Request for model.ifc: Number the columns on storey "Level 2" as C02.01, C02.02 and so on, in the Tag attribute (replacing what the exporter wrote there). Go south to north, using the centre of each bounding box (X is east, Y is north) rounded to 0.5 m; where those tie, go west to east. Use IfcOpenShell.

First a look at what the model holds.

```python
import ifcopenshell
import ifcopenshell.util.element
import ifcopenshell.util.placement

model = ifcopenshell.open("model.ifc")
print(model.schema)
storey = next(s for s in model.by_type("IfcBuildingStorey") if s.Name == "Level 2")
columns = [e for e in ifcopenshell.util.element.get_decomposition(storey) if e.is_a("IfcColumn")]
for e in sorted(columns, key=lambda e: e.id()):
    origin = ifcopenshell.util.placement.get_local_placement(e.ObjectPlacement)[:3, 3]
    print(e.id(), e.Tag, e.Name, origin.round(2) + 0.0, sep=" | ")
```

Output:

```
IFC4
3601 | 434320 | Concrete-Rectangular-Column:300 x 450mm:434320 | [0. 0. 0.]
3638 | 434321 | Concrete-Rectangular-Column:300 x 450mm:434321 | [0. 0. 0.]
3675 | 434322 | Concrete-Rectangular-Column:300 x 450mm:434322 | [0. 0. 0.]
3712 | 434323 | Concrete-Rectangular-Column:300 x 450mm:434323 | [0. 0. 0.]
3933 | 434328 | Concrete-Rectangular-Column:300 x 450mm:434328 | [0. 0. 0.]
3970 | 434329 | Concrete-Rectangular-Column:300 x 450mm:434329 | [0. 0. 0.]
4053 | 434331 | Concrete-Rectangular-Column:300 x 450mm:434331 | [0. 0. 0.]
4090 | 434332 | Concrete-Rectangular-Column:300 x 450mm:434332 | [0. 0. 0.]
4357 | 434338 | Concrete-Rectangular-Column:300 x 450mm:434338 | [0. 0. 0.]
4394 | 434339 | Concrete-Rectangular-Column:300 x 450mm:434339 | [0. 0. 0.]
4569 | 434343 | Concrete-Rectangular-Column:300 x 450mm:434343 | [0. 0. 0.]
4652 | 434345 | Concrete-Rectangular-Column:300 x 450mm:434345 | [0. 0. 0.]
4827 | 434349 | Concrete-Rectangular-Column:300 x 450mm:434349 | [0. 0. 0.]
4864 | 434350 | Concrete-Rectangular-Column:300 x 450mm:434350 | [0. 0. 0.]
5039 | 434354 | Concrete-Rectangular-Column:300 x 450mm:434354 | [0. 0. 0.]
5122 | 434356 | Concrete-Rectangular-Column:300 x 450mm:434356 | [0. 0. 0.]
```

```python
import ifcopenshell
import ifcopenshell.geom
import ifcopenshell.util.element
import ifcopenshell.util.shape

model = ifcopenshell.open("model.ifc")
settings = ifcopenshell.geom.settings()
settings.set("use-world-coords", True)


def centre(element):
    shape = ifcopenshell.geom.create_shape(settings, element)
    return ifcopenshell.util.shape.get_bbox_centroid(shape.geometry)


storey = next(s for s in model.by_type("IfcBuildingStorey") if s.Name == "Level 2")
columns = [e for e in ifcopenshell.util.element.get_decomposition(storey) if e.is_a("IfcColumn")]

# Insertion points can sit at a corner or the storey origin, so sort by the geometry (in metres).
centres = {e: centre(e) for e in columns}
columns.sort(key=lambda e: (round(centres[e][1] / 0.5), centres[e][0]))

for i, e in enumerate(columns, start=1):
    number = f"C02.{i:02d}"
    e.Tag = number
    print(e.id(), number)

model.write("model_updated.ifc")
```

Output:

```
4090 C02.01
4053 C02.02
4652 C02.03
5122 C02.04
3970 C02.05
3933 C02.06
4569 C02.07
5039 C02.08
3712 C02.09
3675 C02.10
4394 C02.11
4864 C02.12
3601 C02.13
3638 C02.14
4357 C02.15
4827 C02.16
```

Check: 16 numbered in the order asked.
